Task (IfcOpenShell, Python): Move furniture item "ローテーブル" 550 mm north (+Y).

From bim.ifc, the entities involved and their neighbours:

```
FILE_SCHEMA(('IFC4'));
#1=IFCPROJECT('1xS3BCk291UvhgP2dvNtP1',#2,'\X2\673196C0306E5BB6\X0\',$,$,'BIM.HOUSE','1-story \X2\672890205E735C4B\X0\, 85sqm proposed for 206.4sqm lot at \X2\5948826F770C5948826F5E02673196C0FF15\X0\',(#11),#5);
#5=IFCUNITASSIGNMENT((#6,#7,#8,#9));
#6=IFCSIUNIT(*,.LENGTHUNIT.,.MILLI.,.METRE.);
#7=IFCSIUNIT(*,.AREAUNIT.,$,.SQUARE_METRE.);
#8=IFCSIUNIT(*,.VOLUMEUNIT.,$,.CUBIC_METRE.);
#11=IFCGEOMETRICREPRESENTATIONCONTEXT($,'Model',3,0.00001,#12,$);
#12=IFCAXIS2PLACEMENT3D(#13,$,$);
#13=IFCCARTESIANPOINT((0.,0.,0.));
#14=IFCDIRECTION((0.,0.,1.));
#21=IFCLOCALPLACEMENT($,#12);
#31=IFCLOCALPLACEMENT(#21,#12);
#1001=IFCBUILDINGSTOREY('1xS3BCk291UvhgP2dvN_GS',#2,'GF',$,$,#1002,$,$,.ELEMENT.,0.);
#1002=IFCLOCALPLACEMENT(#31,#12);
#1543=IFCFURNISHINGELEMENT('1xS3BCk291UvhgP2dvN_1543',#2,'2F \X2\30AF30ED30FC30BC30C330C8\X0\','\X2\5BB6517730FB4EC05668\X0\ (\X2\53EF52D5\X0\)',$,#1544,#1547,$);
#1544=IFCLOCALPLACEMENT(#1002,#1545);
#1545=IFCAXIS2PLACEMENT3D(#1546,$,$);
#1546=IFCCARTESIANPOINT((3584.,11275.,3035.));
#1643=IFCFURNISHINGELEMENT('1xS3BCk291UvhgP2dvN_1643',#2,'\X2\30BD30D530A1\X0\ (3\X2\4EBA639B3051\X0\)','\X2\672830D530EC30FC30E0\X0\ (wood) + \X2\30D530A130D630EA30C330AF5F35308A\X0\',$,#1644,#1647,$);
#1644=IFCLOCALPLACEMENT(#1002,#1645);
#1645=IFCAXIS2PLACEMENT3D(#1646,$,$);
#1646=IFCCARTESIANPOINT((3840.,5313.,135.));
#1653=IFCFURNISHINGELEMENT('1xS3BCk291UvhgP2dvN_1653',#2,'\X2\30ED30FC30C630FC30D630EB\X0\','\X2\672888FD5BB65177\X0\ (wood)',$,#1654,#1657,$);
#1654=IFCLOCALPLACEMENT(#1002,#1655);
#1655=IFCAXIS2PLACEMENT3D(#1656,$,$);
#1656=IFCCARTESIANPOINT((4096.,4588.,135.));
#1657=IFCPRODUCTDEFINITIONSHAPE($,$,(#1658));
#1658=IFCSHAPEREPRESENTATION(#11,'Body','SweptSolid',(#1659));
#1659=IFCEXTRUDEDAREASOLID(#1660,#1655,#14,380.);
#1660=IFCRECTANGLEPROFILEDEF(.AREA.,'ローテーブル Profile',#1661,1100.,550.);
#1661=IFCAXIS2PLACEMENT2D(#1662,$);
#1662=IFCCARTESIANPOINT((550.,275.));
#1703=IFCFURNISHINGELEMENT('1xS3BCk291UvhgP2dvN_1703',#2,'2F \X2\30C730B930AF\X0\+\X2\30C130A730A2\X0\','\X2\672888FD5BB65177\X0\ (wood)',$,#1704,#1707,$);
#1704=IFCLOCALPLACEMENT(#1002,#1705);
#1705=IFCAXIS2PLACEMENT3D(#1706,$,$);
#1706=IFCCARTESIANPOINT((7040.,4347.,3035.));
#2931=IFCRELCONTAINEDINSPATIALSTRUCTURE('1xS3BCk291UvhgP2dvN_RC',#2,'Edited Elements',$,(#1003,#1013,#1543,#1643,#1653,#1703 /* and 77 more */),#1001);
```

```python
import ifcopenshell
import ifcopenshell.api.geometry
import ifcopenshell.util.placement
import ifcopenshell.util.unit

model = ifcopenshell.open("bim.ifc")
unit_scale = ifcopenshell.util.unit.calculate_unit_scale(model)

item = model.by_id(1653)
matrix = ifcopenshell.util.placement.get_local_placement(item.ObjectPlacement)
matrix[1, 3] += 0.55 / unit_scale
ifcopenshell.api.geometry.edit_object_placement(model, product=item, matrix=matrix, is_si=False)

print(ifcopenshell.util.placement.get_local_placement(item.ObjectPlacement).round(3) + 0.0)

model.write("bim_rev.ifc")
```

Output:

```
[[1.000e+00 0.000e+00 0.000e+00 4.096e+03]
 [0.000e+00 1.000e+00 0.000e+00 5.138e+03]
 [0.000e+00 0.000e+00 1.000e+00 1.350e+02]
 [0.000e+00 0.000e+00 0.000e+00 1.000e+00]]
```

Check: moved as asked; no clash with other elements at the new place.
